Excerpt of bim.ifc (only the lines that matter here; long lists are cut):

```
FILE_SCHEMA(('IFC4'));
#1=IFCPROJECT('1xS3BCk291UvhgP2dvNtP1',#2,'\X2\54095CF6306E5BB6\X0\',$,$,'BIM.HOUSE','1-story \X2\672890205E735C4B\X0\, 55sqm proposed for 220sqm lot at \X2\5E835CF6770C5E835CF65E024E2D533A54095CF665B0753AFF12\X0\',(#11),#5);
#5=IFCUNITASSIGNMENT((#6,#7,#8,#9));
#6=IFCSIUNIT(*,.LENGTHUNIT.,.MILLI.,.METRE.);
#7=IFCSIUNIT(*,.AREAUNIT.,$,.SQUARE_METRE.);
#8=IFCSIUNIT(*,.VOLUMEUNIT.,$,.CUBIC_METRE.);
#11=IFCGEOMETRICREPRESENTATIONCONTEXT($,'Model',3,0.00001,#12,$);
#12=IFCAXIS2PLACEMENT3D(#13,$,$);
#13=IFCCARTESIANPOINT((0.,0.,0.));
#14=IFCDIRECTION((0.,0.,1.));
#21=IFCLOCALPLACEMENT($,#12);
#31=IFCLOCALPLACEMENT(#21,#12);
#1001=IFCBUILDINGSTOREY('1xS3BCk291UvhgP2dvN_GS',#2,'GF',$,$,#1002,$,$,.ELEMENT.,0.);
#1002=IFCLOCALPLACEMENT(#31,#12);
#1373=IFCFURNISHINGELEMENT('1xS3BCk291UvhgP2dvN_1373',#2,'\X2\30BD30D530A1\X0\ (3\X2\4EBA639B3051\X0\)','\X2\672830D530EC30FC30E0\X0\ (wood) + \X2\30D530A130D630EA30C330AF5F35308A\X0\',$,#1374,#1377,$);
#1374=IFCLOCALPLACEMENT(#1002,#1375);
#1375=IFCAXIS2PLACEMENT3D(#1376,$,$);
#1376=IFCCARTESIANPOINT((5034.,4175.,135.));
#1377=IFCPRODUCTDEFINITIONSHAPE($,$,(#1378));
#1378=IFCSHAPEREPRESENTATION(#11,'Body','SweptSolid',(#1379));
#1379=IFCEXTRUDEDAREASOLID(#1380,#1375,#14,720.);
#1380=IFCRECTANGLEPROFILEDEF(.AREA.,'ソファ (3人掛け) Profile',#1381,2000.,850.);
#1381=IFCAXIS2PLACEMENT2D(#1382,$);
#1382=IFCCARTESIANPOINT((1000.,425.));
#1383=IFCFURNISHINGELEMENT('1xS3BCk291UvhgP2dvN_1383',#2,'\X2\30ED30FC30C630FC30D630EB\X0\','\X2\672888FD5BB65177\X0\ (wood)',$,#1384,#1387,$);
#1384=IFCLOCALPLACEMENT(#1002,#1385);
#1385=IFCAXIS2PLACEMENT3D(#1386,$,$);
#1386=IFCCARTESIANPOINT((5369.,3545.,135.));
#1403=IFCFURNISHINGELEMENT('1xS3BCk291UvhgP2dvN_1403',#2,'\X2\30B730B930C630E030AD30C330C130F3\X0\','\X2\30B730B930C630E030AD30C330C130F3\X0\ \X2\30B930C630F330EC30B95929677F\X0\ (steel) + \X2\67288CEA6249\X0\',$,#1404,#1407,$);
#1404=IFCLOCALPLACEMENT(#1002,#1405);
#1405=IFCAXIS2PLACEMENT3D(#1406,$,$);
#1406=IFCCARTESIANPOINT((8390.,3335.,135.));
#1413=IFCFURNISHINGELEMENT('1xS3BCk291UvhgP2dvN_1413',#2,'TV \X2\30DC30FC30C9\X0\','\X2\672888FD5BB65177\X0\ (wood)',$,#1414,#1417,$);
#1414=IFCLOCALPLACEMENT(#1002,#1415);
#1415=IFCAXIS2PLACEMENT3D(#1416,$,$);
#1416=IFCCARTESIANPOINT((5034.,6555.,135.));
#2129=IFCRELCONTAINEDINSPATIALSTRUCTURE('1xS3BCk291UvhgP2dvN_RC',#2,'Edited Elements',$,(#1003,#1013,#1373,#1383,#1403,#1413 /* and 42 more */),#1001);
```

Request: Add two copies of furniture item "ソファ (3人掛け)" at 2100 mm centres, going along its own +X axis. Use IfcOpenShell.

```python
import ifcopenshell
import ifcopenshell.api.geometry
import ifcopenshell.api.root
import ifcopenshell.util.element
import ifcopenshell.util.placement

model = ifcopenshell.open("bim.ifc")


def reuse_history(source, copy):
    """copy_class also copies each property set's owner history, people and application; keep the originals."""
    for rel in copy.IsDefinedBy:
        if rel.is_a("IfcRelDefinesByProperties") and (history := rel.RelatingPropertyDefinition.OwnerHistory):
            rel.RelatingPropertyDefinition.OwnerHistory = source.OwnerHistory
            ifcopenshell.util.element.remove_deep2(model, history)


source = model.by_guid("1xS3BCk291UvhgP2dvN_1373")
base = ifcopenshell.util.placement.get_local_placement(source.ObjectPlacement)
step = base[:3, 0] * 2100.0

for i in range(1, 3):
    copy = ifcopenshell.api.root.copy_class(model, product=source)
    copy.Representation = ifcopenshell.util.element.copy_deep(
        model, source.Representation, exclude=["IfcGeometricRepresentationContext", "IfcRepresentationMap"]
    )
    reuse_history(source, copy)
    matrix = base.copy()
    matrix[:3, 3] += i * step
    print("added at", matrix[:3, 3].round(3) + 0.0)
    ifcopenshell.api.geometry.edit_object_placement(model, product=copy, matrix=matrix, is_si=False)

model.write("bim_edited.ifc")
```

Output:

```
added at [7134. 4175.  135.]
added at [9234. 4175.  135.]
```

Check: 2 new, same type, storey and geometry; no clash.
